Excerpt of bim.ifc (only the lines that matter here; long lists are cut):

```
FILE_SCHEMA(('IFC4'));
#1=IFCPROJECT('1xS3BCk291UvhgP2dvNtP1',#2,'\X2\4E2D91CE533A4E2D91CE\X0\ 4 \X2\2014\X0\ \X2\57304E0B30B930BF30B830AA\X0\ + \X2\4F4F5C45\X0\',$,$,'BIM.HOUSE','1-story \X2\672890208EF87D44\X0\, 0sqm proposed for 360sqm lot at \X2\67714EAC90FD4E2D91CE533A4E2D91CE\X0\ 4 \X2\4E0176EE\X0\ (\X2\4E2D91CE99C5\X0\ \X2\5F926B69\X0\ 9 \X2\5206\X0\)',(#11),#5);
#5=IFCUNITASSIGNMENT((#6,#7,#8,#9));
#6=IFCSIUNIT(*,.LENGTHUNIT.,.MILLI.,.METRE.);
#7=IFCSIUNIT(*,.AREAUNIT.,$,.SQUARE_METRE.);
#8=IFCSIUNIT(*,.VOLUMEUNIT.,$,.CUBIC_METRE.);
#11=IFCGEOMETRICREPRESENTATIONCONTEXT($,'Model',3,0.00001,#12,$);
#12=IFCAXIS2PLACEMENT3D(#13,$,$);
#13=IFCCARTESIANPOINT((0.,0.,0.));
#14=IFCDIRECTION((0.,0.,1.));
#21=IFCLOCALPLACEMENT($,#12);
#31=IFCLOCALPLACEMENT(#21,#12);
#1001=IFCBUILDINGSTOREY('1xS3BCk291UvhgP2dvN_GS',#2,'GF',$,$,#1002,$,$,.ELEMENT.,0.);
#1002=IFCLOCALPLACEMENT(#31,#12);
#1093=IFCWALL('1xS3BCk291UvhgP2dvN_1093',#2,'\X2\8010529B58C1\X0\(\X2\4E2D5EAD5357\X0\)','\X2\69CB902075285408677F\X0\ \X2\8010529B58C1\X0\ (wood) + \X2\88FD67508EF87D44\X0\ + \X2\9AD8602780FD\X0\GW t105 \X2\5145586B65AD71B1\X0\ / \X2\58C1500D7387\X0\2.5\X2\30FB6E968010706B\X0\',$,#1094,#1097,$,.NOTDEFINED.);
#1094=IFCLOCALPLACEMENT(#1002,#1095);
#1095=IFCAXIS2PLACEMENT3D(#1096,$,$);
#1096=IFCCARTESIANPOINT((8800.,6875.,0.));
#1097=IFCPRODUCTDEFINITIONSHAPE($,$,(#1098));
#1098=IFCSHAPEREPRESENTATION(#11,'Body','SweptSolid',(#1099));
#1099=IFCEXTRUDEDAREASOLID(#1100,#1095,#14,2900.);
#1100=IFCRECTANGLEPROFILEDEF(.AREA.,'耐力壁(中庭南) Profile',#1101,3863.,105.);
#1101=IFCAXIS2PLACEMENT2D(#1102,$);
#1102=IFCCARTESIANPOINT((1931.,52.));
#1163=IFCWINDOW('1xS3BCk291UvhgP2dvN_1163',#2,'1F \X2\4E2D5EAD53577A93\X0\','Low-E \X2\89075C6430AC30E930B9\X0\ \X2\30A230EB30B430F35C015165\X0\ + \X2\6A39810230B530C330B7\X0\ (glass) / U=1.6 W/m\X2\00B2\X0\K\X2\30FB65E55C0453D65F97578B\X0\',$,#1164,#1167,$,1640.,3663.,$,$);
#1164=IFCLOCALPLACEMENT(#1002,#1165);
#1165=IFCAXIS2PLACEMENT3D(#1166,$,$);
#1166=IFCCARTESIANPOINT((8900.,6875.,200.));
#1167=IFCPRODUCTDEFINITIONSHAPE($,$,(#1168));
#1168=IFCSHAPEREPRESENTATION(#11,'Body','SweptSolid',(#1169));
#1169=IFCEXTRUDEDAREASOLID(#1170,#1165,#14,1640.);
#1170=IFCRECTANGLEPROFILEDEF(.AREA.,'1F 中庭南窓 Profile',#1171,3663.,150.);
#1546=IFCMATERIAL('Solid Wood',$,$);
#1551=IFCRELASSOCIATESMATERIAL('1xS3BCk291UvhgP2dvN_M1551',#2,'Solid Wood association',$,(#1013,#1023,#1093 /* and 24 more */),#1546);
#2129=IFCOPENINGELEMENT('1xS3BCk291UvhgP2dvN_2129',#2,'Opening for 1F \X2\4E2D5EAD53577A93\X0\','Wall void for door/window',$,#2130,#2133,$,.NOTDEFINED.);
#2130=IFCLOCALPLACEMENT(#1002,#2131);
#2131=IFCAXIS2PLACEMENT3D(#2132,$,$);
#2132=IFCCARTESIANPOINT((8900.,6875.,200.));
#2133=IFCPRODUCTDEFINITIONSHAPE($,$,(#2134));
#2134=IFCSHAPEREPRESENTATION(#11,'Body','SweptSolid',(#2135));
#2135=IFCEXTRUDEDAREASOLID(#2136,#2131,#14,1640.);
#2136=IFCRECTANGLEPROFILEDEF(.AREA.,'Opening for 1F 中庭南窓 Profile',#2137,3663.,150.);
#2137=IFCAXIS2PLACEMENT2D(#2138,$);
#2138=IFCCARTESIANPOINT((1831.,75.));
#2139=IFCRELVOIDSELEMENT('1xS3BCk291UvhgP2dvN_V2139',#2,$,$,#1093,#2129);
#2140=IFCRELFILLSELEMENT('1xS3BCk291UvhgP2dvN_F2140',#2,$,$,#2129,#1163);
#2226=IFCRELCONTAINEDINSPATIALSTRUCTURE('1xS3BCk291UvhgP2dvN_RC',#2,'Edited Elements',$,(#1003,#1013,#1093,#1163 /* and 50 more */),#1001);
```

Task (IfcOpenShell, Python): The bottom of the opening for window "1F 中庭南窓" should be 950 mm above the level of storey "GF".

```python
import numpy as np
import ifcopenshell
import ifcopenshell.api.geometry
import ifcopenshell.geom
import ifcopenshell.util.element
import ifcopenshell.util.placement
import ifcopenshell.util.shape
import ifcopenshell.util.unit

model = ifcopenshell.open("bim.ifc")
unit_scale = ifcopenshell.util.unit.calculate_unit_scale(model)

window = model.by_guid("1xS3BCk291UvhgP2dvN_1163")
opening = window.FillsVoids[0].RelatingOpeningElement
storey = ifcopenshell.util.element.get_container(window, ifc_class="IfcBuildingStorey")
level = ifcopenshell.util.placement.get_local_placement(storey.ObjectPlacement)[2, 3]

# The opening's origin need not be at the sill, so measure its lowest point.
shape = ifcopenshell.geom.create_shape(ifcopenshell.geom.settings(), opening)
bottom = ifcopenshell.util.shape.get_shape_bottom_elevation(shape, shape.geometry) / unit_scale
dz = level + 0.95 / unit_scale - bottom

shift = np.array([0.0, 0.0, dz])
# The window is not placed relative to its opening, so move both.
for product in (opening, window):
    matrix = ifcopenshell.util.placement.get_local_placement(product.ObjectPlacement)
    matrix[:3, 3] += shift
    ifcopenshell.api.geometry.edit_object_placement(model, product=product, matrix=matrix, is_si=False)

print(f"moved by {dz * unit_scale:+.3f} m")

model.write("bim_rev.ifc")
```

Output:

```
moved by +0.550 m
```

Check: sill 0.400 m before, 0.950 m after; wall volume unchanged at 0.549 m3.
